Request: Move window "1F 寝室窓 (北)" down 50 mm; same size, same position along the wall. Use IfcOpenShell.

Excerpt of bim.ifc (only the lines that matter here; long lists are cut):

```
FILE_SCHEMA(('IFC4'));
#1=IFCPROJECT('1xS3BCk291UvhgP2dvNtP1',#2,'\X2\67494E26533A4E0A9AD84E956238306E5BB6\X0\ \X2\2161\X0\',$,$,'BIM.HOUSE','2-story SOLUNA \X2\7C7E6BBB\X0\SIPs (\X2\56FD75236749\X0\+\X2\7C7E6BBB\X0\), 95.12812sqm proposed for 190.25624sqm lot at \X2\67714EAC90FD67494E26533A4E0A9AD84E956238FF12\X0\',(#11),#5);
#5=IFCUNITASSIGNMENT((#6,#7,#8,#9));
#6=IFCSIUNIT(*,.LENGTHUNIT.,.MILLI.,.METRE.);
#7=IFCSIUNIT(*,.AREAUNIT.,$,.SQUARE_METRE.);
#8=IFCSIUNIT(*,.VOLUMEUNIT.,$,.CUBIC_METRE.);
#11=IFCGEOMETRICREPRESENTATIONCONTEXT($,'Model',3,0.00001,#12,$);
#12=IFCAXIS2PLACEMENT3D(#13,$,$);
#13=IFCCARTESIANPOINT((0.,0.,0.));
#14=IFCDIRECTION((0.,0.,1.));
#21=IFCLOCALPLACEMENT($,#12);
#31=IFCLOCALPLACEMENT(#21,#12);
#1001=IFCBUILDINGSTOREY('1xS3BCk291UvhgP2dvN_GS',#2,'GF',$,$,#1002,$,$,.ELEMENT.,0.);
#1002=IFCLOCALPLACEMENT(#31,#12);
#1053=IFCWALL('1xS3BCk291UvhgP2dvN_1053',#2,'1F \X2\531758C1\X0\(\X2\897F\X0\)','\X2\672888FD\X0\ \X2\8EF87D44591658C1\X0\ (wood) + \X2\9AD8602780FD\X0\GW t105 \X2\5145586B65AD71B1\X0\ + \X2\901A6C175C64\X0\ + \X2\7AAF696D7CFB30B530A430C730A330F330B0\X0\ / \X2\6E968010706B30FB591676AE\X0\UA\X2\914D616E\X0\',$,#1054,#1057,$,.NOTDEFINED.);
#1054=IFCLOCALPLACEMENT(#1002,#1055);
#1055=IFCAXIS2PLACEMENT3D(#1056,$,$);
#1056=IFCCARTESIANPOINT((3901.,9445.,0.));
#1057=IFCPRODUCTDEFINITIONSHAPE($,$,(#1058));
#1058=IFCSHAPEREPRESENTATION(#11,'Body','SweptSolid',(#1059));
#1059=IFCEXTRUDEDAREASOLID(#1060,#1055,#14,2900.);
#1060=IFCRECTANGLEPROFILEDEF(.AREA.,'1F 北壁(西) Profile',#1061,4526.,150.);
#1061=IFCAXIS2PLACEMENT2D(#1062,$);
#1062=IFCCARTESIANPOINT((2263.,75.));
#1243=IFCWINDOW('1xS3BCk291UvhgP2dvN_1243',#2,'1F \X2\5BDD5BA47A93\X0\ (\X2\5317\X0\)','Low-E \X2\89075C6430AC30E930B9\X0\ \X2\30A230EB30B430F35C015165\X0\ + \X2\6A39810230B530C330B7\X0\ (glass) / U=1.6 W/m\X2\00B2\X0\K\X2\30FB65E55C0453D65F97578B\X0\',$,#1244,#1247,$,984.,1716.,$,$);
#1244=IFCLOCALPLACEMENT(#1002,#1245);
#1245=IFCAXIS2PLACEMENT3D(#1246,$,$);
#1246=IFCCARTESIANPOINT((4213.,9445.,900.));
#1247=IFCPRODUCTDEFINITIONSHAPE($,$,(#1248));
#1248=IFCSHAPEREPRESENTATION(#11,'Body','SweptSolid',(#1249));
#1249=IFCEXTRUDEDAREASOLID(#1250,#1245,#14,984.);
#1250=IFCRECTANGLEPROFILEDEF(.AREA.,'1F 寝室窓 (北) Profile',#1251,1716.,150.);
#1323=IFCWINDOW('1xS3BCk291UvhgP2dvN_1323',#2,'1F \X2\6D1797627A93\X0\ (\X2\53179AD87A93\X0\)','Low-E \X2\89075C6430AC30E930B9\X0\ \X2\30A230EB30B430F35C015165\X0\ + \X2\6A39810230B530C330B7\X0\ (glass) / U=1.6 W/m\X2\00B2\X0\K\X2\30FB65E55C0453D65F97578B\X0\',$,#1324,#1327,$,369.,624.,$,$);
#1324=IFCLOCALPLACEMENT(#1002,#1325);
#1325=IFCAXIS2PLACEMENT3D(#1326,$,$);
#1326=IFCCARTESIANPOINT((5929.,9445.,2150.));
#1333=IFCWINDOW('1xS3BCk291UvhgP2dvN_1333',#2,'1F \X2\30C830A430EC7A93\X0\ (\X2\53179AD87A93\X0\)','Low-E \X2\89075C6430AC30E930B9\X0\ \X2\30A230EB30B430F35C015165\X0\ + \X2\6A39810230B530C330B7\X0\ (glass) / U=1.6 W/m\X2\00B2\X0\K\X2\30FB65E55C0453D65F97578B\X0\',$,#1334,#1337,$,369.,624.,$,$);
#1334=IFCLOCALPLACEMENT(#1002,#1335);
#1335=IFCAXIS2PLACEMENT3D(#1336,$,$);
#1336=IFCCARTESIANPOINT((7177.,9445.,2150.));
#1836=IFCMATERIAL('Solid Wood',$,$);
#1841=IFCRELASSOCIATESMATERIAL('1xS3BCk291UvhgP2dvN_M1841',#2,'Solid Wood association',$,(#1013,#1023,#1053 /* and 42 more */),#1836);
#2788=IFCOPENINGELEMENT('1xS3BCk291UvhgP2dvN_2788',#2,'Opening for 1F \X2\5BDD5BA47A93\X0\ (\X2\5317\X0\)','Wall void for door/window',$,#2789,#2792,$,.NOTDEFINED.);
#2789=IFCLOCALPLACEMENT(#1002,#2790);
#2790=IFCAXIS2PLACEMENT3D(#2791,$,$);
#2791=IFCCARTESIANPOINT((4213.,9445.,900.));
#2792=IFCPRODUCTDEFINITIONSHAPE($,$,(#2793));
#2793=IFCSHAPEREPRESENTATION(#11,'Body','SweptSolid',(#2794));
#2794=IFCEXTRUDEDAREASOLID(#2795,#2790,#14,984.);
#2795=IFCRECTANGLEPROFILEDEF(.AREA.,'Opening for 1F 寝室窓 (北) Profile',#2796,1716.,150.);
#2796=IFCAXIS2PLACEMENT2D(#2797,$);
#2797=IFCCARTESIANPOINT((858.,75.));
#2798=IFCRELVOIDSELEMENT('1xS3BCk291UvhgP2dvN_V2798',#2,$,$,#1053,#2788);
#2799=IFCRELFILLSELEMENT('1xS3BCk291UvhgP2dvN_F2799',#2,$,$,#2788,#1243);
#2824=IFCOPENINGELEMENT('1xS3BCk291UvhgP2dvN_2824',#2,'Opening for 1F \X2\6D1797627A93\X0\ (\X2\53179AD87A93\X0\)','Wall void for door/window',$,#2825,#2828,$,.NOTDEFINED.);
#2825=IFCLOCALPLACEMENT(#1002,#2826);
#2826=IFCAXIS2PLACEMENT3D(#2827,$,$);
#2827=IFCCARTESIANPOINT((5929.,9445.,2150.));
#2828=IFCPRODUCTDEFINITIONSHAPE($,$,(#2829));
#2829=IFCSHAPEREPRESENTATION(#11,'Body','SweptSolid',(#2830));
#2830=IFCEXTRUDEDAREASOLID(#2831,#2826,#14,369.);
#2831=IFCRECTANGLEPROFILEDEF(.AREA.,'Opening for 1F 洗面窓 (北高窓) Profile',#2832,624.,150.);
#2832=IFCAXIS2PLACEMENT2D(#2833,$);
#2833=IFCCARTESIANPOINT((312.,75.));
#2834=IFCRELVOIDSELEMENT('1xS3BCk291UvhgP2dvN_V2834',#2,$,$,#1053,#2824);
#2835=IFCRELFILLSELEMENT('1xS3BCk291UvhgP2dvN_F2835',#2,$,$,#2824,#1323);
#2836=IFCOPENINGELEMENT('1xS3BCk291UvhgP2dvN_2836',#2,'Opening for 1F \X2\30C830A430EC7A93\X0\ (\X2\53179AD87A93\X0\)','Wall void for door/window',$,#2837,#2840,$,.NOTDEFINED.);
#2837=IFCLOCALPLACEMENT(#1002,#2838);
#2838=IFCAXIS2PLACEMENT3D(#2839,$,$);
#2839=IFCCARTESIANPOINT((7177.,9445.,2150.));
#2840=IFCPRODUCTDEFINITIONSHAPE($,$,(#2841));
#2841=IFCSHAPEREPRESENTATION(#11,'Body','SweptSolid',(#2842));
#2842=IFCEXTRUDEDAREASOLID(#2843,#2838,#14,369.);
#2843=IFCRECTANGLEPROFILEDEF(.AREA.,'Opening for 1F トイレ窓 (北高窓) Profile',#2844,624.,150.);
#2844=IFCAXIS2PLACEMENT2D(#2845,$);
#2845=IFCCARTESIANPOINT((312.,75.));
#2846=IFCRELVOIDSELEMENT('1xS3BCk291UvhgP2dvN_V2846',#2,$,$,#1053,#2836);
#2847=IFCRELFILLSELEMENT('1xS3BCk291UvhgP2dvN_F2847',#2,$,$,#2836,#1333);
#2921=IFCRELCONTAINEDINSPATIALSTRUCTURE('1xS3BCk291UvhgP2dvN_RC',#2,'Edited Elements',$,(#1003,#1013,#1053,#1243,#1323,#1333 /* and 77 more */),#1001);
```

```python
import numpy as np
import ifcopenshell
import ifcopenshell.api.geometry
import ifcopenshell.util.placement
import ifcopenshell.util.unit

model = ifcopenshell.open("bim.ifc")
unit_scale = ifcopenshell.util.unit.calculate_unit_scale(model)

window = model.by_guid("1xS3BCk291UvhgP2dvN_1243")
opening = window.FillsVoids[0].RelatingOpeningElement
dz = -50.0

shift = np.array([0.0, 0.0, dz])
# The window is not placed relative to its opening, so move both.
for product in (opening, window):
    matrix = ifcopenshell.util.placement.get_local_placement(product.ObjectPlacement)
    matrix[:3, 3] += shift
    ifcopenshell.api.geometry.edit_object_placement(model, product=product, matrix=matrix, is_si=False)

print(f"moved by {dz * unit_scale:+.3f} m")

model.write("bim_rev.ifc")
```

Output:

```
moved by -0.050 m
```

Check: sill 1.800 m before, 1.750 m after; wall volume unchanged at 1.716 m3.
